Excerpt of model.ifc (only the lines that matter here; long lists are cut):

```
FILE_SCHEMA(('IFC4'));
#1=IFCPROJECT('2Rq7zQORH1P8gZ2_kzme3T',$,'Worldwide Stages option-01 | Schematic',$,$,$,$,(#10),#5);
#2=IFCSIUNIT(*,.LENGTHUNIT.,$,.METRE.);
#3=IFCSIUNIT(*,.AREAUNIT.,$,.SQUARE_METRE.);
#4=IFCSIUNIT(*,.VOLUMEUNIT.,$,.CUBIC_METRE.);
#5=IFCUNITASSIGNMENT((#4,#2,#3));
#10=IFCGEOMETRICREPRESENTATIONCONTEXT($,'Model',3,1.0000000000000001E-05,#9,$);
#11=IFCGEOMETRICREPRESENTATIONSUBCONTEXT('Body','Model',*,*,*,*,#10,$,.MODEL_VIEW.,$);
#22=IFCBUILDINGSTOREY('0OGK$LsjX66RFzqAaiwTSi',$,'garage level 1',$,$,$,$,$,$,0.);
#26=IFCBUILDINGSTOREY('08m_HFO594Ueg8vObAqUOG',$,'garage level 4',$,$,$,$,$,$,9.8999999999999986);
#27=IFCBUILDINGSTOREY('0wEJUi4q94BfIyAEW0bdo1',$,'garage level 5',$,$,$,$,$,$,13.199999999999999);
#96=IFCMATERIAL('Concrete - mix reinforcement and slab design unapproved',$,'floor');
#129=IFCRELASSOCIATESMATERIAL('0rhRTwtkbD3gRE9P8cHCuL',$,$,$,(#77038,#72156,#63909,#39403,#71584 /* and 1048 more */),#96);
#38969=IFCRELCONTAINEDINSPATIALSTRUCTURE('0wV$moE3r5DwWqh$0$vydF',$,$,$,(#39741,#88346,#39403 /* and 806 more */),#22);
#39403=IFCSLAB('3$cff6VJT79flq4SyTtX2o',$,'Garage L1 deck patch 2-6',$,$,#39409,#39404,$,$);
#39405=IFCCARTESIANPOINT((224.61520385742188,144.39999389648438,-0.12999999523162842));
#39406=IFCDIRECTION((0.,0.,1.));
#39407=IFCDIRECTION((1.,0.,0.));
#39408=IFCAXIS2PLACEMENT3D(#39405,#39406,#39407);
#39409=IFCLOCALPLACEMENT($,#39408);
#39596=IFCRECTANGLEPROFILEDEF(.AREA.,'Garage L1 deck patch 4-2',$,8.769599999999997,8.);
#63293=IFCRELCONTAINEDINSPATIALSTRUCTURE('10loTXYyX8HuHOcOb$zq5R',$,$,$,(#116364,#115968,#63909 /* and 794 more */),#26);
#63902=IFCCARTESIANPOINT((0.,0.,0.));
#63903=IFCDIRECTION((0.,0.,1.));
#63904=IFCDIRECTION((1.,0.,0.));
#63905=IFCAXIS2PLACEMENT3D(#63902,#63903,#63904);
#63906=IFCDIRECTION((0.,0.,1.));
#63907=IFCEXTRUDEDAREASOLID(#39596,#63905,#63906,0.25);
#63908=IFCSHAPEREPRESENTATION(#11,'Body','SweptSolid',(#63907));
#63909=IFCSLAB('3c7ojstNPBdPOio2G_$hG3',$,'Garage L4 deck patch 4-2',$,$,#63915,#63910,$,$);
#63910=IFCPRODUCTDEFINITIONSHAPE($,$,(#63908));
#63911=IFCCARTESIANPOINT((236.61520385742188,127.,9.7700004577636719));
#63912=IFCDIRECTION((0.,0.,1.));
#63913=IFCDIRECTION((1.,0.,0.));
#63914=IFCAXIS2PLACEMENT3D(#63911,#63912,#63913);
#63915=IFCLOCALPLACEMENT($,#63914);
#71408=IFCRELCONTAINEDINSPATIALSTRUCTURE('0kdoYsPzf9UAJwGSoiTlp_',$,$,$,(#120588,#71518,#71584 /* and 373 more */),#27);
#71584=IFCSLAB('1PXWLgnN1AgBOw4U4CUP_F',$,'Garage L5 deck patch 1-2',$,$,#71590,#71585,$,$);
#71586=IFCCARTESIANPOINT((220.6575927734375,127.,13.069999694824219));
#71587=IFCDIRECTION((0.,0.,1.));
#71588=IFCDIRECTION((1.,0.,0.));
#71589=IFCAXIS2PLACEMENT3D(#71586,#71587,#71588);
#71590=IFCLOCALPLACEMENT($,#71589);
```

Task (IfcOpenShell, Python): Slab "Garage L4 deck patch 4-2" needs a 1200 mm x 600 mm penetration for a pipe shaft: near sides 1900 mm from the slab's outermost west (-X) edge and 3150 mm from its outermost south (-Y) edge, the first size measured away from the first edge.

```python
import numpy as np
import ifcopenshell
import ifcopenshell.api.feature
import ifcopenshell.api.geometry
import ifcopenshell.api.root
import ifcopenshell.geom
import ifcopenshell.util.placement
import ifcopenshell.util.representation
import ifcopenshell.util.shape
import ifcopenshell.util.unit

model = ifcopenshell.open("model.ifc")
unit_scale = ifcopenshell.util.unit.calculate_unit_scale(model)
settings = ifcopenshell.geom.settings()


def volume(element):
    """Net volume in cubic metres, openings subtracted."""
    shape = ifcopenshell.geom.create_shape(settings, element)
    return ifcopenshell.util.shape.get_volume(shape.geometry)


slab = model.by_guid("3c7ojstNPBdPOio2G_$hG3")
before = volume(slab)

# Extent in the slab's own axes, in metres. The edges named are its -X and -Y sides.
slab_shape = ifcopenshell.geom.create_shape(settings, slab)
vertices = ifcopenshell.util.shape.get_vertices(slab_shape.geometry)
x_min, y_min, bottom = vertices.min(axis=0)
top = vertices[:, 2].max()

opening = ifcopenshell.api.root.create_entity(model, ifc_class="IfcOpeningElement", name="Pipe shaft opening", predefined_type="OPENING")
context = ifcopenshell.util.representation.get_context(model, "Model", "Body", "MODEL_VIEW")
width, depth = 1.2, 0.6
outline = [(0.0, 0.0), (width, 0.0), (width, depth), (0.0, depth), (0.0, 0.0)]
# Overshoot both faces by 50 mm so the cut is clean.
shape = ifcopenshell.api.geometry.add_slab_representation(
    model, context=context, depth=top - bottom + 0.1, polyline=outline
)
ifcopenshell.api.geometry.assign_representation(model, product=opening, representation=shape)

matrix = ifcopenshell.util.placement.get_local_placement(slab.ObjectPlacement)
matrix[:, 3] = matrix @ np.append(np.array([x_min + 1.9, y_min + 3.15, bottom - 0.05]) / unit_scale, 1.0)
ifcopenshell.api.geometry.edit_object_placement(model, product=opening, matrix=matrix, is_si=False)
ifcopenshell.api.feature.add_feature(model, feature=opening, element=slab)

after = volume(slab)

print(f"slab volume {before:.3f} -> {after:.3f} m3")

model.write("model_updated.ifc")
```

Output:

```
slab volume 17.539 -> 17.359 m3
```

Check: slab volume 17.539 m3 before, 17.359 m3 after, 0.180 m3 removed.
